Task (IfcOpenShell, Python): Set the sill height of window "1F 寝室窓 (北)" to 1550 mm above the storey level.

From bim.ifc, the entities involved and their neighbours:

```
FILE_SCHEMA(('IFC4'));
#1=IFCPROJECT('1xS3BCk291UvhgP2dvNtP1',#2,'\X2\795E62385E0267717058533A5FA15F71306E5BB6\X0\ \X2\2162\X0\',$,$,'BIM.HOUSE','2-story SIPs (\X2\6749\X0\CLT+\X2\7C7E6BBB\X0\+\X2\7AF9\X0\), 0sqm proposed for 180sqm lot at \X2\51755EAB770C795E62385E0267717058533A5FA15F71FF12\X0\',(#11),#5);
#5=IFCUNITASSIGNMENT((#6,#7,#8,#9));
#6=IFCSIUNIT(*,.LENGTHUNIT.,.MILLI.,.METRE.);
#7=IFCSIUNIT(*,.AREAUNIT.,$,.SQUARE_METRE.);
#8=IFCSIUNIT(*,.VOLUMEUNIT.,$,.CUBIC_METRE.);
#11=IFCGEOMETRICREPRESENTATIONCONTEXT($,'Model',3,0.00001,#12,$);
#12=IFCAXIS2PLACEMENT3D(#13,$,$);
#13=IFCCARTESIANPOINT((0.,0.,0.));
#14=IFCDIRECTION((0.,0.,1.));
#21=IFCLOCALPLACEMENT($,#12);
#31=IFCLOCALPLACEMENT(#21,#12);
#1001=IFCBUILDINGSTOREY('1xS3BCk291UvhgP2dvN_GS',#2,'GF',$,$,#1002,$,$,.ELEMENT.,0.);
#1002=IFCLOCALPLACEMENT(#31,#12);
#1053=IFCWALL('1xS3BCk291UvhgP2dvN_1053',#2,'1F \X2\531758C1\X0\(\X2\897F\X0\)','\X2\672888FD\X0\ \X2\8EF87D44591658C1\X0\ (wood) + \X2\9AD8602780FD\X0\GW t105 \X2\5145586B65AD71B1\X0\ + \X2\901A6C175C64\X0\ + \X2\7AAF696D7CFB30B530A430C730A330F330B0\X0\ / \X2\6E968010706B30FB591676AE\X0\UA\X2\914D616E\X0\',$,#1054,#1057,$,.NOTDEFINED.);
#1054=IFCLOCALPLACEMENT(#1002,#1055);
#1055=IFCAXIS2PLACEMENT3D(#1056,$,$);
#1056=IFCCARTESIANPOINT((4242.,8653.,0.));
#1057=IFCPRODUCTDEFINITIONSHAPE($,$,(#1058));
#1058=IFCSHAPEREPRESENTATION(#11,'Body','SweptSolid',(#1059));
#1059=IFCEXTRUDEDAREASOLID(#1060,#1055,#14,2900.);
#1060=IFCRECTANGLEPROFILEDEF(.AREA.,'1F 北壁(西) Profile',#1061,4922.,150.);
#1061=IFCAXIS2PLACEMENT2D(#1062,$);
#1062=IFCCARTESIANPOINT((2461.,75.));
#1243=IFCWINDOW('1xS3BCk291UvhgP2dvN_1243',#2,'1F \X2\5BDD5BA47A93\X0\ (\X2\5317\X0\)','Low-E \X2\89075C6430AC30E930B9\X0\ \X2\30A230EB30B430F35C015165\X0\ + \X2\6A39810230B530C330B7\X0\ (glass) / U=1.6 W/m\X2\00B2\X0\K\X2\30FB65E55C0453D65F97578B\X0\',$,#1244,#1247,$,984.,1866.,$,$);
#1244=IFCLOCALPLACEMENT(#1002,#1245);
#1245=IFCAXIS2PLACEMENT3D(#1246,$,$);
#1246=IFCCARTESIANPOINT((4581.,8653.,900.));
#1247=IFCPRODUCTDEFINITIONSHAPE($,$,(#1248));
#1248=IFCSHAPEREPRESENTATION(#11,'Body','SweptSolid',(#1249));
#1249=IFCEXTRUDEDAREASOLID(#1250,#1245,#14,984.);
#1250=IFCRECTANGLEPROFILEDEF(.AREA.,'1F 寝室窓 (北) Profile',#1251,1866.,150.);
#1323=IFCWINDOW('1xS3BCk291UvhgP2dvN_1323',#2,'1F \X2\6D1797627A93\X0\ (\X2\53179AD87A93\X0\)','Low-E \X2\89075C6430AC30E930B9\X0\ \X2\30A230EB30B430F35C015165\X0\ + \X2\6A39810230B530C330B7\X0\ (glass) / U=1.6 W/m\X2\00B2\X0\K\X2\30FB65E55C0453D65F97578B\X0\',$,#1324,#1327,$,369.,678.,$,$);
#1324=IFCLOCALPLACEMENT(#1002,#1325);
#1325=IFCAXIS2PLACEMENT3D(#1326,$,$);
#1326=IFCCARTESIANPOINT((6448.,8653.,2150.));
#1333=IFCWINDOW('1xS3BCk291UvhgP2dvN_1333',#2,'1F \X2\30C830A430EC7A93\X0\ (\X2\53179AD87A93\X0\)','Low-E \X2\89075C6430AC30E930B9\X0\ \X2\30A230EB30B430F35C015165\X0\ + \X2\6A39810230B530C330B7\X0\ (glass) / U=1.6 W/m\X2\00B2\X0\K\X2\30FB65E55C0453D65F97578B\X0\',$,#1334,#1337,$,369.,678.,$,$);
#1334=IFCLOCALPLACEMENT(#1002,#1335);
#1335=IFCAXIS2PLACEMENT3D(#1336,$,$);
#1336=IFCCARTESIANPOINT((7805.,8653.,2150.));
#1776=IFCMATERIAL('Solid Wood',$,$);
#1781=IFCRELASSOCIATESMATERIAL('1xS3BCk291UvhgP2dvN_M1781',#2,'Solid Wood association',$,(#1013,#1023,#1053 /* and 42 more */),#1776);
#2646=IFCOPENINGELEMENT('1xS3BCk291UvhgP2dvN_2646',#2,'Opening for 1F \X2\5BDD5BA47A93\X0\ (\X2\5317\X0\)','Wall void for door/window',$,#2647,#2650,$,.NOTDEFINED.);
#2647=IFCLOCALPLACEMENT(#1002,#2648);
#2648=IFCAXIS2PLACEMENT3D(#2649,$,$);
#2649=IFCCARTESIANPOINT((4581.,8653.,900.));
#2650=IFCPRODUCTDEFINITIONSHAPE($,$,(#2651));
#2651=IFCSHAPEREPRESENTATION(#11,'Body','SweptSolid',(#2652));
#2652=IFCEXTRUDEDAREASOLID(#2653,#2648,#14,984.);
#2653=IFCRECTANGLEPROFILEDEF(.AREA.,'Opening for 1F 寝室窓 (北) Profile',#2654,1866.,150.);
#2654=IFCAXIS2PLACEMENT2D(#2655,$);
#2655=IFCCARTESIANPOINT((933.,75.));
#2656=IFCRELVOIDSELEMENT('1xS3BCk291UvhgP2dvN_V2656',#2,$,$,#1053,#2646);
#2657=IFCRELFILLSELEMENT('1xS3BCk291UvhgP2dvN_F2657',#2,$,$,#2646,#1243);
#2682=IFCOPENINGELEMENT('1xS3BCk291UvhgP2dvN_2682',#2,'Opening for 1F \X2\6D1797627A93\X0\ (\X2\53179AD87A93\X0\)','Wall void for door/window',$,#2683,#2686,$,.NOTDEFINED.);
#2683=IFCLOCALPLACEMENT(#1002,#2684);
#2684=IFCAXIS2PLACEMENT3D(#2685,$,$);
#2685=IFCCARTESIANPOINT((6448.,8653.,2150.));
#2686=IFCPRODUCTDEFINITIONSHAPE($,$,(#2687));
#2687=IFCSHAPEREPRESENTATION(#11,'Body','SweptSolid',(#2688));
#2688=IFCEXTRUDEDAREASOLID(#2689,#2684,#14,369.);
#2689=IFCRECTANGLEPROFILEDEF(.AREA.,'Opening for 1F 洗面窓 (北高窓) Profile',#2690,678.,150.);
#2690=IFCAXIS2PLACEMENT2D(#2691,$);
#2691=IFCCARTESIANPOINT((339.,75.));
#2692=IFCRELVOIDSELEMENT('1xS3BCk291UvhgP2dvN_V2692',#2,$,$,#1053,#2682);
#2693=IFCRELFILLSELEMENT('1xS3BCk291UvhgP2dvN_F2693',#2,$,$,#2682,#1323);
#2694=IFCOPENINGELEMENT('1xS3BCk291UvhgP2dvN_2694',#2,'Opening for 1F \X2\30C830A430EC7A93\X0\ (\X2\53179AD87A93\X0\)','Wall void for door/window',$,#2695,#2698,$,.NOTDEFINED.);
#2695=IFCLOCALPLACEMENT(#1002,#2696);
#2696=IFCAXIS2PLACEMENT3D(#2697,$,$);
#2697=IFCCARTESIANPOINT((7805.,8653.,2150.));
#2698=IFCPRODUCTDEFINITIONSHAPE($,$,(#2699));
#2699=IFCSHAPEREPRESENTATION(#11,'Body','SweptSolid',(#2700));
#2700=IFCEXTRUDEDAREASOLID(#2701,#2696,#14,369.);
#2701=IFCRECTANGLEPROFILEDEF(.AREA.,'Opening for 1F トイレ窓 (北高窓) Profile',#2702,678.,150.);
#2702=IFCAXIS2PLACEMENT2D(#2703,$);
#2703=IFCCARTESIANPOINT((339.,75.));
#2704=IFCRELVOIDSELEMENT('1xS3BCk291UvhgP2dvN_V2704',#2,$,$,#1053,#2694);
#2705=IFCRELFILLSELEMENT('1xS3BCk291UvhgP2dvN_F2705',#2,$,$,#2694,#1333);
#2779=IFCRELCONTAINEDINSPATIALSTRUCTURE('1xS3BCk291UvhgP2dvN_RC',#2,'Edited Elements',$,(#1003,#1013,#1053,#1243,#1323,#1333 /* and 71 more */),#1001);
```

```python
import numpy as np
import ifcopenshell
import ifcopenshell.api.geometry
import ifcopenshell.geom
import ifcopenshell.util.element
import ifcopenshell.util.placement
import ifcopenshell.util.shape
import ifcopenshell.util.unit

model = ifcopenshell.open("bim.ifc")
unit_scale = ifcopenshell.util.unit.calculate_unit_scale(model)

window = model.by_guid("1xS3BCk291UvhgP2dvN_1243")
opening = window.FillsVoids[0].RelatingOpeningElement
storey = ifcopenshell.util.element.get_container(window, ifc_class="IfcBuildingStorey")
level = ifcopenshell.util.placement.get_local_placement(storey.ObjectPlacement)[2, 3]

# The opening's origin need not be at the sill, so measure its lowest point.
shape = ifcopenshell.geom.create_shape(ifcopenshell.geom.settings(), opening)
bottom = ifcopenshell.util.shape.get_shape_bottom_elevation(shape, shape.geometry) / unit_scale
dz = level + 1550.0 - bottom

shift = np.array([0.0, 0.0, dz])
# The window is not placed relative to its opening, so move both.
for product in (opening, window):
    matrix = ifcopenshell.util.placement.get_local_placement(product.ObjectPlacement)
    matrix[:3, 3] += shift
    ifcopenshell.api.geometry.edit_object_placement(model, product=product, matrix=matrix, is_si=False)

print(f"moved by {dz * unit_scale:+.3f} m")

model.write("bim_edited.ifc")
```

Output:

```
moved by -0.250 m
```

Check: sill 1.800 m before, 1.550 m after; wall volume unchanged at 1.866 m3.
